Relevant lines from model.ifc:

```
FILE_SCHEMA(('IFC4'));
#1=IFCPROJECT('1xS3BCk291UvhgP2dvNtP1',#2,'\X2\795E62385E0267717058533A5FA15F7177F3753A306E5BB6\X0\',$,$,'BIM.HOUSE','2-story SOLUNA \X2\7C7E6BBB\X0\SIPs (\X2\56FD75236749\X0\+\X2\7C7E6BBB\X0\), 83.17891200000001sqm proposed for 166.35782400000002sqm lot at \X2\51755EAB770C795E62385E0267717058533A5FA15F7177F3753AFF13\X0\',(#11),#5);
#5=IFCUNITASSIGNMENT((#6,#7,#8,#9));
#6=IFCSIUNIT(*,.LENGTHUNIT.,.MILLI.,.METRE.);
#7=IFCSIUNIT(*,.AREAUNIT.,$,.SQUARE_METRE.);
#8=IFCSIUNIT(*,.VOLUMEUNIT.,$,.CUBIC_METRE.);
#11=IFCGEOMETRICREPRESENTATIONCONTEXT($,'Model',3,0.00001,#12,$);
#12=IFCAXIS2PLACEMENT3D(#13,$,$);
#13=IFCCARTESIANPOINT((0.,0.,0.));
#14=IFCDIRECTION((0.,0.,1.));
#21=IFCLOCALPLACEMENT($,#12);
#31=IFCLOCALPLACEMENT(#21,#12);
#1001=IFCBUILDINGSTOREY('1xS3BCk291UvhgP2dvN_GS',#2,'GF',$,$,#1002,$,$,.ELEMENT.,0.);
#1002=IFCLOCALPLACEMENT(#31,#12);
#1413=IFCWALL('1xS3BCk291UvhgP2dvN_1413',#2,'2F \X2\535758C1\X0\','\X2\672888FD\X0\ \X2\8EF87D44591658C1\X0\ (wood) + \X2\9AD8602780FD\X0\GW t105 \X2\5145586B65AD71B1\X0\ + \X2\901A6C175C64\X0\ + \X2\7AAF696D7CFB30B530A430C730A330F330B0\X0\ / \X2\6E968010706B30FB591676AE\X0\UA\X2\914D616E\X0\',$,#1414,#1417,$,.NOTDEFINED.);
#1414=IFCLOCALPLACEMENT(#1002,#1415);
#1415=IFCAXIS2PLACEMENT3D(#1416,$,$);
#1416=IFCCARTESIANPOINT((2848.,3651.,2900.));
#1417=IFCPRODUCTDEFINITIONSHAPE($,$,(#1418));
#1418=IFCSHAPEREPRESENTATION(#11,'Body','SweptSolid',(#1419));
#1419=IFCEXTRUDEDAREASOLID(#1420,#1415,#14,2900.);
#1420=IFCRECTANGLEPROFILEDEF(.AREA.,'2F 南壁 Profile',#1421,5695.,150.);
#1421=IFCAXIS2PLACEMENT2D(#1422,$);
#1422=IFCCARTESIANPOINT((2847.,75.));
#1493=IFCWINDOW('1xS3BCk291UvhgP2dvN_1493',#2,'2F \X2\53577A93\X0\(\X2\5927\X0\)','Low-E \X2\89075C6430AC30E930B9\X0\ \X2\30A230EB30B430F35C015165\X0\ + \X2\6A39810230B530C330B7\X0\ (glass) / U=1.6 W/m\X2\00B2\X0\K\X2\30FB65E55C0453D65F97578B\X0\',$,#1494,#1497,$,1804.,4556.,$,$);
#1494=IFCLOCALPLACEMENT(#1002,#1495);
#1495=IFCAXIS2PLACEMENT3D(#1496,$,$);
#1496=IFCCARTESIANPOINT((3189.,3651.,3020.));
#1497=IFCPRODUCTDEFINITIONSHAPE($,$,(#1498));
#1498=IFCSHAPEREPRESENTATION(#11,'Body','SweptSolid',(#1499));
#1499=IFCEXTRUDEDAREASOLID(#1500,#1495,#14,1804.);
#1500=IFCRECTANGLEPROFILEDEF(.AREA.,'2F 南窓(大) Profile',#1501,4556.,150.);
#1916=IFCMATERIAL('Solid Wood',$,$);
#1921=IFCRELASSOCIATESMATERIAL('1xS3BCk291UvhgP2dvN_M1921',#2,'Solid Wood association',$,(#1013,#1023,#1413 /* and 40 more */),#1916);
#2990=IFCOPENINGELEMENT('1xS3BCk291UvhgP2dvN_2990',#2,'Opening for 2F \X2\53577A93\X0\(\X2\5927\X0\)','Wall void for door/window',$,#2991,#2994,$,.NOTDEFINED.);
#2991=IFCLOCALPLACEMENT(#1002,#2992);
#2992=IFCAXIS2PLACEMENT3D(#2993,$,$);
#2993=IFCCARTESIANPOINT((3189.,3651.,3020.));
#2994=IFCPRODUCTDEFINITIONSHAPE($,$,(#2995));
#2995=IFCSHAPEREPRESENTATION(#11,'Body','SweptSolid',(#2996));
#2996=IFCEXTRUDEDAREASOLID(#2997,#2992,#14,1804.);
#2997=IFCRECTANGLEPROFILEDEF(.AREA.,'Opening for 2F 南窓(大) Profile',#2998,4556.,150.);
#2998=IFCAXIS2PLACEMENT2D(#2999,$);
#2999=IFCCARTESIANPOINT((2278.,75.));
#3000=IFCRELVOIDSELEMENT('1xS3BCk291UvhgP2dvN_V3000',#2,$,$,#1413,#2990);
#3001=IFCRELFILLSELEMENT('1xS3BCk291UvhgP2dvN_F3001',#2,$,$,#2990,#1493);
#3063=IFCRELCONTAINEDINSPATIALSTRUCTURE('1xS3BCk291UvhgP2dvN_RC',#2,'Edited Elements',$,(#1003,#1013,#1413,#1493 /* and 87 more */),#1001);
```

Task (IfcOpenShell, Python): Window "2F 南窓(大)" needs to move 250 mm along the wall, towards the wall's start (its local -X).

```python
import ifcopenshell
import ifcopenshell.api.geometry
import ifcopenshell.util.placement
import ifcopenshell.util.unit

model = ifcopenshell.open("model.ifc")
unit_scale = ifcopenshell.util.unit.calculate_unit_scale(model)

window = model.by_guid("1xS3BCk291UvhgP2dvN_1493")
opening = window.FillsVoids[0].RelatingOpeningElement
wall = opening.VoidsElements[0].RelatingBuildingElement

wall_matrix = ifcopenshell.util.placement.get_local_placement(wall.ObjectPlacement)
shift = wall_matrix[:3, 0] * -0.25 / unit_scale
before = ifcopenshell.util.placement.get_local_placement(window.ObjectPlacement)[:3, 3].copy()

# The window is not placed relative to its opening, so move both.
for product in (opening, window):
    matrix = ifcopenshell.util.placement.get_local_placement(product.ObjectPlacement)
    matrix[:3, 3] += shift
    ifcopenshell.api.geometry.edit_object_placement(model, product=product, matrix=matrix, is_si=False)

after = ifcopenshell.util.placement.get_local_placement(window.ObjectPlacement)[:3, 3]
print("window moved by", (after - before).round(3) + 0.0)

model.write("model_edited.ifc")
```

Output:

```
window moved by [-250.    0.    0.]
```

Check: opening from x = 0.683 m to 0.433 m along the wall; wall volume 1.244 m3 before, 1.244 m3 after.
